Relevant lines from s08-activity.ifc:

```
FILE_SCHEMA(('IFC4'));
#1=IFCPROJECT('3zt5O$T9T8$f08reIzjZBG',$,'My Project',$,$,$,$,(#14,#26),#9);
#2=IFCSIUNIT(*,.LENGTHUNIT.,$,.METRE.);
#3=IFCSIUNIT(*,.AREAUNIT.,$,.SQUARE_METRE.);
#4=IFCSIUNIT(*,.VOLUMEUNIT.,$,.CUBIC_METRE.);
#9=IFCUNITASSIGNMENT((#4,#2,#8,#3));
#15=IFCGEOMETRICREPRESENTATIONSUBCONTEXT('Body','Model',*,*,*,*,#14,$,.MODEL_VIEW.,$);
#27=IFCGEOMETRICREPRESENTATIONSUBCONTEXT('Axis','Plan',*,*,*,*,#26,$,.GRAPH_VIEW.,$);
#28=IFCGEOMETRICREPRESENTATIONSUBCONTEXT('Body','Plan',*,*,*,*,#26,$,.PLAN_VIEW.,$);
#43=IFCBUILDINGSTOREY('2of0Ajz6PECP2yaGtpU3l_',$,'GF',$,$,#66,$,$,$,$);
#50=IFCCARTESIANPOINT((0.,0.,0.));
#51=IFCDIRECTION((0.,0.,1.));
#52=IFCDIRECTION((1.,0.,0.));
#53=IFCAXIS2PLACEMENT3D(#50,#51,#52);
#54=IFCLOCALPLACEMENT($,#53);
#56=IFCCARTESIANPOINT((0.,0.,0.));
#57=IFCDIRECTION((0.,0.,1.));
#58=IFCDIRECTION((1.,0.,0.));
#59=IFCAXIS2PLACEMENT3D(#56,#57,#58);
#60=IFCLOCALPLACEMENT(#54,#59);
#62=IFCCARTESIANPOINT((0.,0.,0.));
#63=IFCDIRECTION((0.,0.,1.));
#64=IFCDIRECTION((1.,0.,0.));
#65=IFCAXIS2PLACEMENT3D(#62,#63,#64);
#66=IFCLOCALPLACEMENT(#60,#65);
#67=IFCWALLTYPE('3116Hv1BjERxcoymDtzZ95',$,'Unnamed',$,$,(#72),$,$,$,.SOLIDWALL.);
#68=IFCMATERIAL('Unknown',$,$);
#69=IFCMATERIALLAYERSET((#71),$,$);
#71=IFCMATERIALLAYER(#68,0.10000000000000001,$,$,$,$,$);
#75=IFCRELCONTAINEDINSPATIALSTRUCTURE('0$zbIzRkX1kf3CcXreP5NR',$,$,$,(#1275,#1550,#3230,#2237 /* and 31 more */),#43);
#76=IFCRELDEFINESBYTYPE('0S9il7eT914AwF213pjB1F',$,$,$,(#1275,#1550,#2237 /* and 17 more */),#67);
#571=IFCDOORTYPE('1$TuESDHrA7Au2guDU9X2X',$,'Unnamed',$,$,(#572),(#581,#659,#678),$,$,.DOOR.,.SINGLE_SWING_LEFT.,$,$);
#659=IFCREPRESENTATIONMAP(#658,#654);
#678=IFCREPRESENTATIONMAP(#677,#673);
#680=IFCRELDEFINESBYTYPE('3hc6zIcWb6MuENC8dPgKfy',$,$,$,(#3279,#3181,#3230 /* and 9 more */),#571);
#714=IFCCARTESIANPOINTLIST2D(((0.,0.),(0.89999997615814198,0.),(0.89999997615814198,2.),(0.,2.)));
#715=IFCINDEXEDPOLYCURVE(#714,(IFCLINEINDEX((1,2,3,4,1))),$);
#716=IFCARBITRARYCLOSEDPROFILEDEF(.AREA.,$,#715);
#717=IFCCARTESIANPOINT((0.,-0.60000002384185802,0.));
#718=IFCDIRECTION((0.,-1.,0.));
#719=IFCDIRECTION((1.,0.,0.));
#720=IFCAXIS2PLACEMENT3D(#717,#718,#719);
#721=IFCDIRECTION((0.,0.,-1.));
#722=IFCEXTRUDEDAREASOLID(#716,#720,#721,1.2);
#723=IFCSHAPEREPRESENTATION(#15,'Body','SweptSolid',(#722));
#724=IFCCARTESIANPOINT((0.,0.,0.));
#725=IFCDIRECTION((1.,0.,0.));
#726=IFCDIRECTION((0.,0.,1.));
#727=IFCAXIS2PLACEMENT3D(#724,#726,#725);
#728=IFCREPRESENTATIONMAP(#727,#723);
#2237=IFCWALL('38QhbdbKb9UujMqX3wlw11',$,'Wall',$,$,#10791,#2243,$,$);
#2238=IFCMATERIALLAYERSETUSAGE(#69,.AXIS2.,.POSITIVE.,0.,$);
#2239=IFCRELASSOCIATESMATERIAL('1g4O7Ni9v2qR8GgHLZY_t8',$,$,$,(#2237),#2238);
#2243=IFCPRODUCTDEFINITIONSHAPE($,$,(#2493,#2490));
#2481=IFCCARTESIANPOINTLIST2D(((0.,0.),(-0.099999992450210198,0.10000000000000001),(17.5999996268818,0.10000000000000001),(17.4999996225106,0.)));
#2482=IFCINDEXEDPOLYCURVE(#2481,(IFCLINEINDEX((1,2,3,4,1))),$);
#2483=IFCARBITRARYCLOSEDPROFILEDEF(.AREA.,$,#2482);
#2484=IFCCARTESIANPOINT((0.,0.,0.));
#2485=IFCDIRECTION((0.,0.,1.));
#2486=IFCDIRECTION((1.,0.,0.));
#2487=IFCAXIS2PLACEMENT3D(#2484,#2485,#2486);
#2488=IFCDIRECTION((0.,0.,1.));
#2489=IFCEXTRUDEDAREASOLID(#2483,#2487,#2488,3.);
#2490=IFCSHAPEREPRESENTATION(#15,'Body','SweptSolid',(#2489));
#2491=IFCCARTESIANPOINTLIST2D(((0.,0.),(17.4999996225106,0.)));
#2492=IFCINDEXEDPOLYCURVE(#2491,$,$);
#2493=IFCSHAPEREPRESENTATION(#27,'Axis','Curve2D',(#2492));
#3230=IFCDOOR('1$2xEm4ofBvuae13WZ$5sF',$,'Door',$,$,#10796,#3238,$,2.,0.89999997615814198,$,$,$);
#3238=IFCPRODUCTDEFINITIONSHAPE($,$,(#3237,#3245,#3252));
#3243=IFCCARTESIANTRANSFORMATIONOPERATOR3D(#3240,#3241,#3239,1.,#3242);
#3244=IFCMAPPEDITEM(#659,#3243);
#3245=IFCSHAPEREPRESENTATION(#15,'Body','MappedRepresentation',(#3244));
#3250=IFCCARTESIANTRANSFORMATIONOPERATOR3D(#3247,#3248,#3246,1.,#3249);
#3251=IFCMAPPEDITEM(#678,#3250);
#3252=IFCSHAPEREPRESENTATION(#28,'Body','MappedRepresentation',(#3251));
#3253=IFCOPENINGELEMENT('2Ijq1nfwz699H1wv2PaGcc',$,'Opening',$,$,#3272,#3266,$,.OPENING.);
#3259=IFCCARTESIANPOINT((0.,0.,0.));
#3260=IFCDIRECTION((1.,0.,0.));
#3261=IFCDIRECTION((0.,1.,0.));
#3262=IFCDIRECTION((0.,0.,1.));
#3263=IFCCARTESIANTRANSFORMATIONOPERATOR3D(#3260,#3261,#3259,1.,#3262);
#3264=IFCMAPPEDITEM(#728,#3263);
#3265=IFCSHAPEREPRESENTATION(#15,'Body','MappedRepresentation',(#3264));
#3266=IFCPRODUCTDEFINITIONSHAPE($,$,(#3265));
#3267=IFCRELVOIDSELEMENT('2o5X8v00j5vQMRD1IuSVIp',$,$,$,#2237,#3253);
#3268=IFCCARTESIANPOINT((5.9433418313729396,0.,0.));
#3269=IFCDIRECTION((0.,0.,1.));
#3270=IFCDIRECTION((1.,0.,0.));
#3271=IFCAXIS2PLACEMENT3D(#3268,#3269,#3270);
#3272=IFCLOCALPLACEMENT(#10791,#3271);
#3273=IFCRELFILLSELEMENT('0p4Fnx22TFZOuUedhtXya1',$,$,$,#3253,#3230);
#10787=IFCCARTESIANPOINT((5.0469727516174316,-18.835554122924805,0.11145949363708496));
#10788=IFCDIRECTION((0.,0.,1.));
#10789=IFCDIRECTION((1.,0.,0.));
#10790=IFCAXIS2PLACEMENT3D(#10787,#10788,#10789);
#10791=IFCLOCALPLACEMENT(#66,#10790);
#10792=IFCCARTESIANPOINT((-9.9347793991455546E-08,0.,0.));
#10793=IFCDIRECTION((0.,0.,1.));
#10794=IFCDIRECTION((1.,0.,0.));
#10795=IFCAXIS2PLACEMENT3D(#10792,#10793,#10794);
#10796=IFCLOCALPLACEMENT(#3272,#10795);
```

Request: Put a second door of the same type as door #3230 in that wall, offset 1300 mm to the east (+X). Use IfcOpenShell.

```python
import ifcopenshell
import ifcopenshell.api.feature
import ifcopenshell.api.geometry
import ifcopenshell.api.root
import ifcopenshell.geom
import ifcopenshell.util.element
import ifcopenshell.util.placement
import ifcopenshell.util.shape
import ifcopenshell.util.unit

model = ifcopenshell.open("s08-activity.ifc")
unit_scale = ifcopenshell.util.unit.calculate_unit_scale(model)
settings = ifcopenshell.geom.settings()


def volume(element):
    """Net volume in cubic metres, openings subtracted."""
    shape = ifcopenshell.geom.create_shape(settings, element)
    return ifcopenshell.util.shape.get_volume(shape.geometry)


door = model.by_guid("1$2xEm4ofBvuae13WZ$5sF")
opening = door.FillsVoids[0].RelatingOpeningElement
wall = opening.VoidsElements[0].RelatingBuildingElement
before = volume(wall)
shift = ifcopenshell.util.placement.get_local_placement(wall.ObjectPlacement)[:3, 0] * 1.3 / unit_scale

# copy_class copies the void relationship, type, container and properties, but no geometry.
new_opening = ifcopenshell.api.root.copy_class(model, product=opening)
new_opening.Representation = ifcopenshell.util.element.copy_deep(
    model, opening.Representation, exclude=["IfcGeometricRepresentationContext", "IfcRepresentationMap"]
)
new_door = ifcopenshell.api.root.copy_class(model, product=door)
new_door.Representation = ifcopenshell.util.element.copy_deep(
    model, door.Representation, exclude=["IfcGeometricRepresentationContext", "IfcRepresentationMap"]
)
ifcopenshell.api.feature.add_filling(model, opening=new_opening, element=new_door)

for old, new in ((opening, new_opening), (door, new_door)):
    matrix = ifcopenshell.util.placement.get_local_placement(old.ObjectPlacement)
    matrix[:3, 3] += shift
    ifcopenshell.api.geometry.edit_object_placement(model, product=new, matrix=matrix, is_si=False)

after = volume(wall)

print(f"wall volume {before:.3f} -> {after:.3f} m3")

model.write("s08-activity-out.ifc")
```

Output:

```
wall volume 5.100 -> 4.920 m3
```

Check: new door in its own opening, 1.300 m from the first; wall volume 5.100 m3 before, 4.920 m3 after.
